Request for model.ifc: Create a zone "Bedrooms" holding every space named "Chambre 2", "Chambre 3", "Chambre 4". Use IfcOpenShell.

First a look at what the model holds.

```python
import ifcopenshell

model = ifcopenshell.open("model.ifc")
print(model.schema)
seen = {}
for space in model.by_type("IfcSpace"):
    seen[space.LongName] = seen.get(space.LongName, 0) + 1
for name, count in sorted(seen.items(), key=str):
    print(count, "x", name)
print("zones:", [z.Name for z in model.by_type("IfcZone")][:20])
```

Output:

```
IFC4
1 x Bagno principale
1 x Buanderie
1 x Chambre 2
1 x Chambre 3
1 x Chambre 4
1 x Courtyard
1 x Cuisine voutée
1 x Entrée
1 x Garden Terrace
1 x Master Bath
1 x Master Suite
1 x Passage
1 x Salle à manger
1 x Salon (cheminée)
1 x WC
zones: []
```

```python
import ifcopenshell
import ifcopenshell.api.group
import ifcopenshell.api.root

model = ifcopenshell.open("model.ifc")

names = {"Chambre 2", "Chambre 3", "Chambre 4"}
spaces = [s for s in model.by_type("IfcSpace") if s.LongName in names]

zone = ifcopenshell.api.root.create_entity(model, ifc_class="IfcZone", name="Bedrooms")
ifcopenshell.api.group.assign_group(model, products=spaces, group=zone)
print(len(spaces), "spaces in", zone.Name)

model.write("model_v2.ifc")
```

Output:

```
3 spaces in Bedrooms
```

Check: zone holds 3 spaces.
